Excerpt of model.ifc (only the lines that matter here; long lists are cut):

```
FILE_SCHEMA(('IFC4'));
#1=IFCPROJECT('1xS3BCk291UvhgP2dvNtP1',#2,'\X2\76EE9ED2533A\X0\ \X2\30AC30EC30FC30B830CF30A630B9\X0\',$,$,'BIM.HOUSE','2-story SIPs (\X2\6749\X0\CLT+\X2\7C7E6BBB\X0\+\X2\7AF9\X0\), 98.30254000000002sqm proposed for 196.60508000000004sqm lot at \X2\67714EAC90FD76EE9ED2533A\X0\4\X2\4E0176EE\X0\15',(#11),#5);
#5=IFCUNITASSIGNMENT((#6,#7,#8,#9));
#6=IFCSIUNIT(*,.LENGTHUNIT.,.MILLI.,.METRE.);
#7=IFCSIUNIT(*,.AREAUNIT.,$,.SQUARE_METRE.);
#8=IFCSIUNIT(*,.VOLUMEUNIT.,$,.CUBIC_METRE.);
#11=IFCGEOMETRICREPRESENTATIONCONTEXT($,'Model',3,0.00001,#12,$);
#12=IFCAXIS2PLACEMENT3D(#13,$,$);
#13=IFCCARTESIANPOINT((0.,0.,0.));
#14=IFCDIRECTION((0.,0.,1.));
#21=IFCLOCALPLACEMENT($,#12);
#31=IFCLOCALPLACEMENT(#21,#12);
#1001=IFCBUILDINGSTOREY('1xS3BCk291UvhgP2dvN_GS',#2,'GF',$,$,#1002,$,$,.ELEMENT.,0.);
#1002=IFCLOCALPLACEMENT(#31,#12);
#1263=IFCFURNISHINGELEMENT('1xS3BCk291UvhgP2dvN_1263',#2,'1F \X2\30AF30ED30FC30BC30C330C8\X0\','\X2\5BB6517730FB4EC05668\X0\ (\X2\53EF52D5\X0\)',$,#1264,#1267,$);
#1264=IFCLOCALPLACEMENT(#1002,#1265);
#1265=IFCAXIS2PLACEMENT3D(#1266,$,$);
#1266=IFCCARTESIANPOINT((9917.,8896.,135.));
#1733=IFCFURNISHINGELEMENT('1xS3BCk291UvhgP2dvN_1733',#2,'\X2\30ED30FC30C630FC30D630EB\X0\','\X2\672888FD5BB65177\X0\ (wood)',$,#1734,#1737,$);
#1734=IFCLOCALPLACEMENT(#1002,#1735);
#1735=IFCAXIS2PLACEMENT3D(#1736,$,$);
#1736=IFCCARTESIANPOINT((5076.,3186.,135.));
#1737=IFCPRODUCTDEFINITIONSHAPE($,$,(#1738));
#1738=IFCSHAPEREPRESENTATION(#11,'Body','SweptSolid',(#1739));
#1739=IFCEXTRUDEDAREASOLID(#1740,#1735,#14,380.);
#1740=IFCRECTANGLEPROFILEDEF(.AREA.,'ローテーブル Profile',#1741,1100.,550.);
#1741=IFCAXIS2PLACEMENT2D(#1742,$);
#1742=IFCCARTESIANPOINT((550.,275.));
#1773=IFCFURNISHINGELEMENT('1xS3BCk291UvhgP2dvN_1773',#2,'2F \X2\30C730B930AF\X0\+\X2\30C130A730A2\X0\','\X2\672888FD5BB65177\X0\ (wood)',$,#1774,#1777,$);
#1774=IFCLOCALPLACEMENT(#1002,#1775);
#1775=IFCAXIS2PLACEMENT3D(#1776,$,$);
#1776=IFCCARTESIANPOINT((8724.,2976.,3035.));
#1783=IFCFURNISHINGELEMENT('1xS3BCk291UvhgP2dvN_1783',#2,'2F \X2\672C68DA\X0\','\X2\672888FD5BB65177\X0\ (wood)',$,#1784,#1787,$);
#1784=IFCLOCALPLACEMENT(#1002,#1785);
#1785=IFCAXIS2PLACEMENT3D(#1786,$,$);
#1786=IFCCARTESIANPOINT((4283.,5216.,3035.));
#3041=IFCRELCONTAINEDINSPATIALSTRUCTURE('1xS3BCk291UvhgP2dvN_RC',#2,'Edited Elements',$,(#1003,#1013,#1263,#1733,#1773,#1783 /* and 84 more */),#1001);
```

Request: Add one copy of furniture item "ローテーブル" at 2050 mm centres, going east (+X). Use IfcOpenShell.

```python
import numpy as np
import ifcopenshell
import ifcopenshell.api.geometry
import ifcopenshell.api.root
import ifcopenshell.util.element
import ifcopenshell.util.placement
import ifcopenshell.util.unit

model = ifcopenshell.open("model.ifc")
unit_scale = ifcopenshell.util.unit.calculate_unit_scale(model)


def reuse_history(source, copy):
    """copy_class also copies each property set's owner history, people and application; keep the originals."""
    for rel in copy.IsDefinedBy:
        if rel.is_a("IfcRelDefinesByProperties") and (history := rel.RelatingPropertyDefinition.OwnerHistory):
            rel.RelatingPropertyDefinition.OwnerHistory = source.OwnerHistory
            ifcopenshell.util.element.remove_deep2(model, history)


source = model.by_guid("1xS3BCk291UvhgP2dvN_1733")
base = ifcopenshell.util.placement.get_local_placement(source.ObjectPlacement)
step = np.array([1.0, 0.0, 0.0]) * 2.05 / unit_scale

for i in range(1, 2):
    copy = ifcopenshell.api.root.copy_class(model, product=source)
    copy.Representation = ifcopenshell.util.element.copy_deep(
        model, source.Representation, exclude=["IfcGeometricRepresentationContext", "IfcRepresentationMap"]
    )
    reuse_history(source, copy)
    matrix = base.copy()
    matrix[:3, 3] += i * step
    print("added at", matrix[:3, 3].round(3) + 0.0)
    ifcopenshell.api.geometry.edit_object_placement(model, product=copy, matrix=matrix, is_si=False)

model.write("model_rev.ifc")
```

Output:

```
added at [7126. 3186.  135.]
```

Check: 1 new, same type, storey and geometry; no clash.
